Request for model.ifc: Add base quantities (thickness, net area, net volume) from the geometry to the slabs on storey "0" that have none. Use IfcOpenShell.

First a look at what the model holds.

```python
import ifcopenshell
import ifcopenshell.util.element
import ifcopenshell.util.unit

model = ifcopenshell.open("model.ifc")
print(model.schema)
for unit_type in ("LENGTHUNIT", "AREAUNIT", "VOLUMEUNIT"):
    print(unit_type, ifcopenshell.util.unit.calculate_unit_scale(model, unit_type))
storey = next(s for s in model.by_type("IfcBuildingStorey") if s.Name == "0")
slabs = [e for e in ifcopenshell.util.element.get_decomposition(storey) if e.is_a("IfcSlab")]
for e in sorted(slabs, key=lambda e: e.id()):
    print(e.id(), e.is_a(), e.Name, list(ifcopenshell.util.element.get_psets(e, qtos_only=True)), sep=" | ")
```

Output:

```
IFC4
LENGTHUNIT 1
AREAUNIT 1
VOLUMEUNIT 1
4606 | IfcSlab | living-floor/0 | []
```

```python
import ifcopenshell
import ifcopenshell.api.pset
import ifcopenshell.geom
import ifcopenshell.util.element
import ifcopenshell.util.shape
import ifcopenshell.util.unit

model = ifcopenshell.open("model.ifc")
unit_scale = ifcopenshell.util.unit.calculate_unit_scale(model)
area_scale = ifcopenshell.util.unit.calculate_unit_scale(model, "AREAUNIT")
volume_scale = ifcopenshell.util.unit.calculate_unit_scale(model, "VOLUMEUNIT")
settings = ifcopenshell.geom.settings()

storey = next(s for s in model.by_type("IfcBuildingStorey") if s.Name == "0")
slabs = [e for e in ifcopenshell.util.element.get_decomposition(storey) if e.is_a("IfcSlab")]

for e in sorted(slabs, key=lambda e: e.id()):
    if ifcopenshell.util.element.get_psets(e, qtos_only=True, should_inherit=False):
        continue
    # Geometry comes back in metres, in the element's own axes.
    shape = ifcopenshell.geom.create_shape(settings, e)
    values = {
        "Width": ifcopenshell.util.shape.get_z(shape.geometry) / unit_scale,
        "NetArea": ifcopenshell.util.shape.get_footprint_area(shape.geometry) / area_scale,
        "NetVolume": ifcopenshell.util.shape.get_volume(shape.geometry) / volume_scale,
    }
    qto = ifcopenshell.api.pset.add_qto(model, product=e, name="Qto_SlabBaseQuantities")
    ifcopenshell.api.pset.edit_qto(model, qto=qto, properties=values)
    print(e.id(), {k: round(v, 3) for k, v in values.items()})

model.write("model_rev.ifc")
```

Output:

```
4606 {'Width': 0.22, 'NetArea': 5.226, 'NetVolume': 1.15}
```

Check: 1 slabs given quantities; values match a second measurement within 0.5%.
